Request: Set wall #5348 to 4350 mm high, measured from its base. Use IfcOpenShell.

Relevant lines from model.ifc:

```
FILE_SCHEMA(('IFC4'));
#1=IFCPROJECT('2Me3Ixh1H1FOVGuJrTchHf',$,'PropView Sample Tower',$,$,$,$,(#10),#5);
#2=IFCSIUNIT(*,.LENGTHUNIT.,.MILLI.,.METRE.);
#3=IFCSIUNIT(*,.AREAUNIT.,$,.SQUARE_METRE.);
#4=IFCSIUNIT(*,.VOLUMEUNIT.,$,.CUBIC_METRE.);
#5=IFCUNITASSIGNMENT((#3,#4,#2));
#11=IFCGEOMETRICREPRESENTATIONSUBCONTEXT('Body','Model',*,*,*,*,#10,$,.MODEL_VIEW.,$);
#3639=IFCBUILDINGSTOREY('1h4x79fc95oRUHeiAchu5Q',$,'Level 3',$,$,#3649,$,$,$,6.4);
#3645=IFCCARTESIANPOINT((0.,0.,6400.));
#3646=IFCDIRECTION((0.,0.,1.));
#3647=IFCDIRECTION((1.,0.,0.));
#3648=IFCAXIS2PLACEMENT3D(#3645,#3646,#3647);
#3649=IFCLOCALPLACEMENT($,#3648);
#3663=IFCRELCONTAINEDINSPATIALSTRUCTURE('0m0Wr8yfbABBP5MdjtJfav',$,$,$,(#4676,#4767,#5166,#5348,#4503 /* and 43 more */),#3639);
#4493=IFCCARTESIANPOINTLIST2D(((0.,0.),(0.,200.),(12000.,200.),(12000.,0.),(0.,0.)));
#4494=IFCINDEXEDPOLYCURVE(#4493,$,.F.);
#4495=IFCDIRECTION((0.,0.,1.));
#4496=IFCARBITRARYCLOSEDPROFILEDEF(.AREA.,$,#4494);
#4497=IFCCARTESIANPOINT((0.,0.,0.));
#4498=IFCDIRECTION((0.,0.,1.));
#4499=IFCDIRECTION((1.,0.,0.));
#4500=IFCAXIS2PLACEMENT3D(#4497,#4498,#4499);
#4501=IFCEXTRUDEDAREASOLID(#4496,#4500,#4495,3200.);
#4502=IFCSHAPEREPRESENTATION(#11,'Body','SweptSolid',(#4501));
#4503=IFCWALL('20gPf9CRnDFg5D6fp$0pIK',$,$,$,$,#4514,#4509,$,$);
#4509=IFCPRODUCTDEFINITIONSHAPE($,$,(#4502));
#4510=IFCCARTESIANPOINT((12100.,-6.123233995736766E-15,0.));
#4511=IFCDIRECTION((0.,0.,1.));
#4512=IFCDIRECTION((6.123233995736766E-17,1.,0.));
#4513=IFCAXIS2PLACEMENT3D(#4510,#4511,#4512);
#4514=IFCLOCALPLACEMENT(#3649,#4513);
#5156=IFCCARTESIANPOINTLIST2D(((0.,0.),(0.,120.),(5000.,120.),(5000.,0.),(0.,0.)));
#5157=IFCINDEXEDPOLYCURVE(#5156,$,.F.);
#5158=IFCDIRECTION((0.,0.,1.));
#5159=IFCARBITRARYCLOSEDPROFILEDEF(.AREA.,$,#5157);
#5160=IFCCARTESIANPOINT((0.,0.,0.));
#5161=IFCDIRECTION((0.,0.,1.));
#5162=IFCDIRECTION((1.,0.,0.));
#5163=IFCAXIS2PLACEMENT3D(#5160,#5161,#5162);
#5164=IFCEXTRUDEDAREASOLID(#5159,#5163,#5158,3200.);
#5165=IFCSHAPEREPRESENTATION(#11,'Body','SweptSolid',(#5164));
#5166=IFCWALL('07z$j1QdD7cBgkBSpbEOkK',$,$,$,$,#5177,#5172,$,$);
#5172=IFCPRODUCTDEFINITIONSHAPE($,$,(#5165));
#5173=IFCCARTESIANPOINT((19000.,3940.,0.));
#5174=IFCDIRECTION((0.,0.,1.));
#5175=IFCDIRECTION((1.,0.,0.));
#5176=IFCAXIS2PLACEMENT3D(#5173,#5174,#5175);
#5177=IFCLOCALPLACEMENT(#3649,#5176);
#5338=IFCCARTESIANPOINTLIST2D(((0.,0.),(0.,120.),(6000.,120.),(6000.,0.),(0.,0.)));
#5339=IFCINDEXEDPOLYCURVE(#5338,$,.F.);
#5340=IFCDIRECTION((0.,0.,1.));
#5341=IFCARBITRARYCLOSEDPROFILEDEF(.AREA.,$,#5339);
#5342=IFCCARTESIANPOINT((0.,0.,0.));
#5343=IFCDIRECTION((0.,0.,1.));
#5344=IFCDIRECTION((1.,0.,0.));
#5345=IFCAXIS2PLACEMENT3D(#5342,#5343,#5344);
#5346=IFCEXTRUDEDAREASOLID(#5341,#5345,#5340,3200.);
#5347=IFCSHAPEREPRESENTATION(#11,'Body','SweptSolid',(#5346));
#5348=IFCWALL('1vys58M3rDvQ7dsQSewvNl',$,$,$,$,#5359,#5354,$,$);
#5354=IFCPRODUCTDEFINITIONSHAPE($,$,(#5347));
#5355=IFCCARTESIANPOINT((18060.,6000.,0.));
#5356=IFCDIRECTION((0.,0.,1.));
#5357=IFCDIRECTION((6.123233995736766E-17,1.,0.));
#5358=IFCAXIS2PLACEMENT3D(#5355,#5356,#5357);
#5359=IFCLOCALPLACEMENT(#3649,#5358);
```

```python
import ifcopenshell
import ifcopenshell.geom
import ifcopenshell.util.representation
import ifcopenshell.util.shape
import ifcopenshell.util.unit

model = ifcopenshell.open("model.ifc")
unit_scale = ifcopenshell.util.unit.calculate_unit_scale(model)
settings = ifcopenshell.geom.settings()


def volume(element):
    """Net volume in cubic metres, openings subtracted."""
    shape = ifcopenshell.geom.create_shape(settings, element)
    return ifcopenshell.util.shape.get_volume(shape.geometry)


wall = model.by_id(5348)
before = volume(wall)

body = ifcopenshell.util.representation.get_representation(wall, "Model", "Body")
solid = body.Items[0]
old_height = solid.Depth
solid.Depth = 4.35 / unit_scale
after = volume(wall)

print(f"height {old_height:g} -> {solid.Depth:g}, volume {before:.3f} -> {after:.3f} m3")

model.write("model_edited.ifc")
```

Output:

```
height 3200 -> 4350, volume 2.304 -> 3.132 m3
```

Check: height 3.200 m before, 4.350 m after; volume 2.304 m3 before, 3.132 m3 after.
